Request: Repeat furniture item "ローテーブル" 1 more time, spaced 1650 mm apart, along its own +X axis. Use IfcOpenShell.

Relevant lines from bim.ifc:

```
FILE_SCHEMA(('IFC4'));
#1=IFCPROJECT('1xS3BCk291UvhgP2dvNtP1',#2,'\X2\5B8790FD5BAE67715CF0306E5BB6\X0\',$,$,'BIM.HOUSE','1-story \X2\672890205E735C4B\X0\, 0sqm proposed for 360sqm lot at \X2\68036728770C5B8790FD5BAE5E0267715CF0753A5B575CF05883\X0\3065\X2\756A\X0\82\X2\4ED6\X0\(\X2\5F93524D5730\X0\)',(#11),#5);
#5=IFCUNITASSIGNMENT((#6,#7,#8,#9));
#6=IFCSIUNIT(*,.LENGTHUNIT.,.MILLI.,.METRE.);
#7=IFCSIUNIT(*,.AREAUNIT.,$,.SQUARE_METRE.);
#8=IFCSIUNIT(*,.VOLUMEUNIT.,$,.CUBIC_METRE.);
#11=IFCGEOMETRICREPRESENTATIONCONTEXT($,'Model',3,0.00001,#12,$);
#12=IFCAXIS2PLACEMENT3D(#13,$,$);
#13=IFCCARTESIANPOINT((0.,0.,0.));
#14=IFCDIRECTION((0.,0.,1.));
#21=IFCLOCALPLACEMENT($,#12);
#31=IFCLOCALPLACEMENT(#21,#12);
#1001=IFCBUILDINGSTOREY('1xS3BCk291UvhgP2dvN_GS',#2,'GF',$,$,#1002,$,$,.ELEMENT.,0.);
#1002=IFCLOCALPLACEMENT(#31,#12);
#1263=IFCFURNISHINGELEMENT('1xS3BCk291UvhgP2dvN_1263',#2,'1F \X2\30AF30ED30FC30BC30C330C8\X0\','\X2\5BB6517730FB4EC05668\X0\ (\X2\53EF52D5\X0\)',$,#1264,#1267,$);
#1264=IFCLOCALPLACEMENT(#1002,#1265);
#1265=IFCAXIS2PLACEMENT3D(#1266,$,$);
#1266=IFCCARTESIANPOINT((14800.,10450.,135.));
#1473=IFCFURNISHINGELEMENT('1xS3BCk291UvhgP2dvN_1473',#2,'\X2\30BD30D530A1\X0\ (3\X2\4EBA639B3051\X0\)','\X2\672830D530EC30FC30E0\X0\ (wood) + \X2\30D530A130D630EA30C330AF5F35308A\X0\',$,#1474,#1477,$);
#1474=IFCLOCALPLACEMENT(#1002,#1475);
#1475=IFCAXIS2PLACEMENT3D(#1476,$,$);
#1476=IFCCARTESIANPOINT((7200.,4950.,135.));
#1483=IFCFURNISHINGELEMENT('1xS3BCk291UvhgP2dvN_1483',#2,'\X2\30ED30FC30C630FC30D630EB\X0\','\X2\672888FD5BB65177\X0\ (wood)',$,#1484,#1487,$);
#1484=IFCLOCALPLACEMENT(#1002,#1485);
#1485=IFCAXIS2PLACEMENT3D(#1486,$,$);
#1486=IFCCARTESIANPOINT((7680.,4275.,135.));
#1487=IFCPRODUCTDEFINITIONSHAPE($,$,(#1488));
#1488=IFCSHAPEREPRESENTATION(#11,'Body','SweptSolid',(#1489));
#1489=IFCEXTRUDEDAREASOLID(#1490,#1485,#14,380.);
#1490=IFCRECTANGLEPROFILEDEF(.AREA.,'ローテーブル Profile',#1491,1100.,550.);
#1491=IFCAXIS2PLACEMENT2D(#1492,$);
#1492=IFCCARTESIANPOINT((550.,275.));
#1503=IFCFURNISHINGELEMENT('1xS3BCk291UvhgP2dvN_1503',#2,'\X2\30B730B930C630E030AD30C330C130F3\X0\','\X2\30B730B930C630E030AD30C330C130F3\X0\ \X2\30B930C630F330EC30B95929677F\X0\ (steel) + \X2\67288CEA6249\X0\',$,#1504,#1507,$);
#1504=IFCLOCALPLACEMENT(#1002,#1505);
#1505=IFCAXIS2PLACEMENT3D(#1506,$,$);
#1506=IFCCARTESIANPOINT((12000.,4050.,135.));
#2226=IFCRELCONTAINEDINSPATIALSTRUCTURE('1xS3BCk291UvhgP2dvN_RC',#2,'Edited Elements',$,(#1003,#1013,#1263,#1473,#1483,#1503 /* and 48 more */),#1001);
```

```python
import ifcopenshell
import ifcopenshell.api.geometry
import ifcopenshell.api.root
import ifcopenshell.util.element
import ifcopenshell.util.placement

model = ifcopenshell.open("bim.ifc")


def reuse_history(source, copy):
    """copy_class also copies each property set's owner history, people and application; keep the originals."""
    for rel in copy.IsDefinedBy:
        if rel.is_a("IfcRelDefinesByProperties") and (history := rel.RelatingPropertyDefinition.OwnerHistory):
            rel.RelatingPropertyDefinition.OwnerHistory = source.OwnerHistory
            ifcopenshell.util.element.remove_deep2(model, history)


source = model.by_id(1483)
base = ifcopenshell.util.placement.get_local_placement(source.ObjectPlacement)
step = base[:3, 0] * 1650.0

for i in range(1, 2):
    copy = ifcopenshell.api.root.copy_class(model, product=source)
    copy.Representation = ifcopenshell.util.element.copy_deep(
        model, source.Representation, exclude=["IfcGeometricRepresentationContext", "IfcRepresentationMap"]
    )
    reuse_history(source, copy)
    matrix = base.copy()
    matrix[:3, 3] += i * step
    print("added at", matrix[:3, 3].round(3) + 0.0)
    ifcopenshell.api.geometry.edit_object_placement(model, product=copy, matrix=matrix, is_si=False)

model.write("bim-out.ifc")
```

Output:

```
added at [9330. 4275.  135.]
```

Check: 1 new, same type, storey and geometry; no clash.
